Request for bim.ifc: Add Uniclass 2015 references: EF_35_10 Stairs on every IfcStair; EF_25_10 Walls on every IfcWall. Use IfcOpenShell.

First a look at what the model holds.

```python
import ifcopenshell

model = ifcopenshell.open("bim.ifc")
print(model.schema)
print("classifications:", [c.Name for c in model.by_type("IfcClassification")])
for ifc_class in ("IfcDoor", "IfcRoof", "IfcStair", "IfcWall", "IfcWindow"):
    print(ifc_class, len(model.by_type(ifc_class)))
```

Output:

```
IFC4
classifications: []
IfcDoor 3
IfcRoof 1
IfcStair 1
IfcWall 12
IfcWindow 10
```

```python
import ifcopenshell
import ifcopenshell.api.classification

model = ifcopenshell.open("bim.ifc")

system = ifcopenshell.api.classification.add_classification(model, classification="Uniclass 2015")

codes = {
    "IfcStair": ("EF_35_10", "Stairs"),
    "IfcWall": ("EF_25_10", "Walls"),
}
for ifc_class, (code, name) in codes.items():
    products = model.by_type(ifc_class)
    ifcopenshell.api.classification.add_reference(
        model, products=products, classification=system, identification=code, name=name
    )
    print(code, len(products))

model.write("bim_v2.ifc")
```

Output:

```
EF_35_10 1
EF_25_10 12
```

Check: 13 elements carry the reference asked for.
